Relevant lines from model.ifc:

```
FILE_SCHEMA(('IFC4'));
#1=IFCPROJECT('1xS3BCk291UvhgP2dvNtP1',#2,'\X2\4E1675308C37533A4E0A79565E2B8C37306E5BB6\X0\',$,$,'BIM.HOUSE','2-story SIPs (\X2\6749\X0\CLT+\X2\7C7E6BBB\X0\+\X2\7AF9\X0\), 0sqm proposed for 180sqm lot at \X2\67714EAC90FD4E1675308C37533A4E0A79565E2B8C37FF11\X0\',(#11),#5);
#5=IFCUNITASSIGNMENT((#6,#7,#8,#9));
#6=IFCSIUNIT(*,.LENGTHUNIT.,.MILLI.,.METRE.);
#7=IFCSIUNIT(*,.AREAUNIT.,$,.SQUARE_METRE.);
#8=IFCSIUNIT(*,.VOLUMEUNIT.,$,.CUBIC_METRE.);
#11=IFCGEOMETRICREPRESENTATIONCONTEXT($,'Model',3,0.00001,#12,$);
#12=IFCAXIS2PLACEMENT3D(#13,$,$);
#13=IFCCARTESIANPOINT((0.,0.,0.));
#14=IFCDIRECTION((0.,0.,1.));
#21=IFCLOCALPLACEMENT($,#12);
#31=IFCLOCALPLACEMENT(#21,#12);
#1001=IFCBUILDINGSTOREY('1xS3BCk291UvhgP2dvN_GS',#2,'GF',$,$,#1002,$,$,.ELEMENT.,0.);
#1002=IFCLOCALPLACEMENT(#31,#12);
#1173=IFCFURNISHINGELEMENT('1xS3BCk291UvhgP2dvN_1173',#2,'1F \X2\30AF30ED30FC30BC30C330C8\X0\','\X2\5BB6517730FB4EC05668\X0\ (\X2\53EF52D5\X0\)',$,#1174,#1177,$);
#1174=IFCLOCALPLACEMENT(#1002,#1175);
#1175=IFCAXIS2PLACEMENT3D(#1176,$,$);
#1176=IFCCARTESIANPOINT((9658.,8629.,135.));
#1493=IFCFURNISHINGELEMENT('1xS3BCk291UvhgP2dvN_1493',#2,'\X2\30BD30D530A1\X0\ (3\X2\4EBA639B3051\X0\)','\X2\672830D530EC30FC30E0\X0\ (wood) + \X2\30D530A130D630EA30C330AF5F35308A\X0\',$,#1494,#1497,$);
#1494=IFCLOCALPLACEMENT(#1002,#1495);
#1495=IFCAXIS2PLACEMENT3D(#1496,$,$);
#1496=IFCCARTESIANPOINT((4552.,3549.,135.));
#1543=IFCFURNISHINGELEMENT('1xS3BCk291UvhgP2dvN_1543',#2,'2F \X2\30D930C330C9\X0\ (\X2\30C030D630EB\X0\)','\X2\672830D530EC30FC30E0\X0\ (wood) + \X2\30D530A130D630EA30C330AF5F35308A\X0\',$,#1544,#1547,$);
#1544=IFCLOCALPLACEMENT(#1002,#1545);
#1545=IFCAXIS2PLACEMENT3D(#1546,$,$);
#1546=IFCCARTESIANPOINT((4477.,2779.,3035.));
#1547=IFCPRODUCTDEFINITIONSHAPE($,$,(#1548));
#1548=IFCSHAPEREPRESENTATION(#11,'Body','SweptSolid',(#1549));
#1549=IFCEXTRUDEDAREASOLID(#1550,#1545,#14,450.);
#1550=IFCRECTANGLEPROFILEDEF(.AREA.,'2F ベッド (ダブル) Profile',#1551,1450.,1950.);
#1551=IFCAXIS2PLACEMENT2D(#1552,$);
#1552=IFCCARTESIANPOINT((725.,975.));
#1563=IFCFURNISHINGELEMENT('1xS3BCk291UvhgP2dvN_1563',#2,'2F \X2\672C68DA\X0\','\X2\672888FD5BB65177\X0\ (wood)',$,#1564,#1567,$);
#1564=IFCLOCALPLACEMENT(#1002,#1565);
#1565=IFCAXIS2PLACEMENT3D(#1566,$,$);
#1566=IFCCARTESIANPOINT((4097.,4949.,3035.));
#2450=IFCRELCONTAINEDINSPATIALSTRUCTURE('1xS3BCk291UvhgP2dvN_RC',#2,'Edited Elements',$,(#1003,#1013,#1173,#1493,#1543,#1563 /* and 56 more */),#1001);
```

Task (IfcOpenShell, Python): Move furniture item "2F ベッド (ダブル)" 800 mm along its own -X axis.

```python
import ifcopenshell
import ifcopenshell.api.geometry
import ifcopenshell.util.placement

model = ifcopenshell.open("model.ifc")

item = model.by_guid("1xS3BCk291UvhgP2dvN_1543")
matrix = ifcopenshell.util.placement.get_local_placement(item.ObjectPlacement)
matrix[:3, 3] -= matrix[:3, 0] * 800.0
ifcopenshell.api.geometry.edit_object_placement(model, product=item, matrix=matrix, is_si=False)

print(ifcopenshell.util.placement.get_local_placement(item.ObjectPlacement).round(3) + 0.0)

model.write("model_edited.ifc")
```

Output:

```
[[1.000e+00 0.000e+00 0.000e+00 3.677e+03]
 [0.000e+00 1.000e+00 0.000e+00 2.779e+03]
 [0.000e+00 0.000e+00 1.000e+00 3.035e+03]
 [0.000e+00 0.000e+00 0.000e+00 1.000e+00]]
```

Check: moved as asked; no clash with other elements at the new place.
